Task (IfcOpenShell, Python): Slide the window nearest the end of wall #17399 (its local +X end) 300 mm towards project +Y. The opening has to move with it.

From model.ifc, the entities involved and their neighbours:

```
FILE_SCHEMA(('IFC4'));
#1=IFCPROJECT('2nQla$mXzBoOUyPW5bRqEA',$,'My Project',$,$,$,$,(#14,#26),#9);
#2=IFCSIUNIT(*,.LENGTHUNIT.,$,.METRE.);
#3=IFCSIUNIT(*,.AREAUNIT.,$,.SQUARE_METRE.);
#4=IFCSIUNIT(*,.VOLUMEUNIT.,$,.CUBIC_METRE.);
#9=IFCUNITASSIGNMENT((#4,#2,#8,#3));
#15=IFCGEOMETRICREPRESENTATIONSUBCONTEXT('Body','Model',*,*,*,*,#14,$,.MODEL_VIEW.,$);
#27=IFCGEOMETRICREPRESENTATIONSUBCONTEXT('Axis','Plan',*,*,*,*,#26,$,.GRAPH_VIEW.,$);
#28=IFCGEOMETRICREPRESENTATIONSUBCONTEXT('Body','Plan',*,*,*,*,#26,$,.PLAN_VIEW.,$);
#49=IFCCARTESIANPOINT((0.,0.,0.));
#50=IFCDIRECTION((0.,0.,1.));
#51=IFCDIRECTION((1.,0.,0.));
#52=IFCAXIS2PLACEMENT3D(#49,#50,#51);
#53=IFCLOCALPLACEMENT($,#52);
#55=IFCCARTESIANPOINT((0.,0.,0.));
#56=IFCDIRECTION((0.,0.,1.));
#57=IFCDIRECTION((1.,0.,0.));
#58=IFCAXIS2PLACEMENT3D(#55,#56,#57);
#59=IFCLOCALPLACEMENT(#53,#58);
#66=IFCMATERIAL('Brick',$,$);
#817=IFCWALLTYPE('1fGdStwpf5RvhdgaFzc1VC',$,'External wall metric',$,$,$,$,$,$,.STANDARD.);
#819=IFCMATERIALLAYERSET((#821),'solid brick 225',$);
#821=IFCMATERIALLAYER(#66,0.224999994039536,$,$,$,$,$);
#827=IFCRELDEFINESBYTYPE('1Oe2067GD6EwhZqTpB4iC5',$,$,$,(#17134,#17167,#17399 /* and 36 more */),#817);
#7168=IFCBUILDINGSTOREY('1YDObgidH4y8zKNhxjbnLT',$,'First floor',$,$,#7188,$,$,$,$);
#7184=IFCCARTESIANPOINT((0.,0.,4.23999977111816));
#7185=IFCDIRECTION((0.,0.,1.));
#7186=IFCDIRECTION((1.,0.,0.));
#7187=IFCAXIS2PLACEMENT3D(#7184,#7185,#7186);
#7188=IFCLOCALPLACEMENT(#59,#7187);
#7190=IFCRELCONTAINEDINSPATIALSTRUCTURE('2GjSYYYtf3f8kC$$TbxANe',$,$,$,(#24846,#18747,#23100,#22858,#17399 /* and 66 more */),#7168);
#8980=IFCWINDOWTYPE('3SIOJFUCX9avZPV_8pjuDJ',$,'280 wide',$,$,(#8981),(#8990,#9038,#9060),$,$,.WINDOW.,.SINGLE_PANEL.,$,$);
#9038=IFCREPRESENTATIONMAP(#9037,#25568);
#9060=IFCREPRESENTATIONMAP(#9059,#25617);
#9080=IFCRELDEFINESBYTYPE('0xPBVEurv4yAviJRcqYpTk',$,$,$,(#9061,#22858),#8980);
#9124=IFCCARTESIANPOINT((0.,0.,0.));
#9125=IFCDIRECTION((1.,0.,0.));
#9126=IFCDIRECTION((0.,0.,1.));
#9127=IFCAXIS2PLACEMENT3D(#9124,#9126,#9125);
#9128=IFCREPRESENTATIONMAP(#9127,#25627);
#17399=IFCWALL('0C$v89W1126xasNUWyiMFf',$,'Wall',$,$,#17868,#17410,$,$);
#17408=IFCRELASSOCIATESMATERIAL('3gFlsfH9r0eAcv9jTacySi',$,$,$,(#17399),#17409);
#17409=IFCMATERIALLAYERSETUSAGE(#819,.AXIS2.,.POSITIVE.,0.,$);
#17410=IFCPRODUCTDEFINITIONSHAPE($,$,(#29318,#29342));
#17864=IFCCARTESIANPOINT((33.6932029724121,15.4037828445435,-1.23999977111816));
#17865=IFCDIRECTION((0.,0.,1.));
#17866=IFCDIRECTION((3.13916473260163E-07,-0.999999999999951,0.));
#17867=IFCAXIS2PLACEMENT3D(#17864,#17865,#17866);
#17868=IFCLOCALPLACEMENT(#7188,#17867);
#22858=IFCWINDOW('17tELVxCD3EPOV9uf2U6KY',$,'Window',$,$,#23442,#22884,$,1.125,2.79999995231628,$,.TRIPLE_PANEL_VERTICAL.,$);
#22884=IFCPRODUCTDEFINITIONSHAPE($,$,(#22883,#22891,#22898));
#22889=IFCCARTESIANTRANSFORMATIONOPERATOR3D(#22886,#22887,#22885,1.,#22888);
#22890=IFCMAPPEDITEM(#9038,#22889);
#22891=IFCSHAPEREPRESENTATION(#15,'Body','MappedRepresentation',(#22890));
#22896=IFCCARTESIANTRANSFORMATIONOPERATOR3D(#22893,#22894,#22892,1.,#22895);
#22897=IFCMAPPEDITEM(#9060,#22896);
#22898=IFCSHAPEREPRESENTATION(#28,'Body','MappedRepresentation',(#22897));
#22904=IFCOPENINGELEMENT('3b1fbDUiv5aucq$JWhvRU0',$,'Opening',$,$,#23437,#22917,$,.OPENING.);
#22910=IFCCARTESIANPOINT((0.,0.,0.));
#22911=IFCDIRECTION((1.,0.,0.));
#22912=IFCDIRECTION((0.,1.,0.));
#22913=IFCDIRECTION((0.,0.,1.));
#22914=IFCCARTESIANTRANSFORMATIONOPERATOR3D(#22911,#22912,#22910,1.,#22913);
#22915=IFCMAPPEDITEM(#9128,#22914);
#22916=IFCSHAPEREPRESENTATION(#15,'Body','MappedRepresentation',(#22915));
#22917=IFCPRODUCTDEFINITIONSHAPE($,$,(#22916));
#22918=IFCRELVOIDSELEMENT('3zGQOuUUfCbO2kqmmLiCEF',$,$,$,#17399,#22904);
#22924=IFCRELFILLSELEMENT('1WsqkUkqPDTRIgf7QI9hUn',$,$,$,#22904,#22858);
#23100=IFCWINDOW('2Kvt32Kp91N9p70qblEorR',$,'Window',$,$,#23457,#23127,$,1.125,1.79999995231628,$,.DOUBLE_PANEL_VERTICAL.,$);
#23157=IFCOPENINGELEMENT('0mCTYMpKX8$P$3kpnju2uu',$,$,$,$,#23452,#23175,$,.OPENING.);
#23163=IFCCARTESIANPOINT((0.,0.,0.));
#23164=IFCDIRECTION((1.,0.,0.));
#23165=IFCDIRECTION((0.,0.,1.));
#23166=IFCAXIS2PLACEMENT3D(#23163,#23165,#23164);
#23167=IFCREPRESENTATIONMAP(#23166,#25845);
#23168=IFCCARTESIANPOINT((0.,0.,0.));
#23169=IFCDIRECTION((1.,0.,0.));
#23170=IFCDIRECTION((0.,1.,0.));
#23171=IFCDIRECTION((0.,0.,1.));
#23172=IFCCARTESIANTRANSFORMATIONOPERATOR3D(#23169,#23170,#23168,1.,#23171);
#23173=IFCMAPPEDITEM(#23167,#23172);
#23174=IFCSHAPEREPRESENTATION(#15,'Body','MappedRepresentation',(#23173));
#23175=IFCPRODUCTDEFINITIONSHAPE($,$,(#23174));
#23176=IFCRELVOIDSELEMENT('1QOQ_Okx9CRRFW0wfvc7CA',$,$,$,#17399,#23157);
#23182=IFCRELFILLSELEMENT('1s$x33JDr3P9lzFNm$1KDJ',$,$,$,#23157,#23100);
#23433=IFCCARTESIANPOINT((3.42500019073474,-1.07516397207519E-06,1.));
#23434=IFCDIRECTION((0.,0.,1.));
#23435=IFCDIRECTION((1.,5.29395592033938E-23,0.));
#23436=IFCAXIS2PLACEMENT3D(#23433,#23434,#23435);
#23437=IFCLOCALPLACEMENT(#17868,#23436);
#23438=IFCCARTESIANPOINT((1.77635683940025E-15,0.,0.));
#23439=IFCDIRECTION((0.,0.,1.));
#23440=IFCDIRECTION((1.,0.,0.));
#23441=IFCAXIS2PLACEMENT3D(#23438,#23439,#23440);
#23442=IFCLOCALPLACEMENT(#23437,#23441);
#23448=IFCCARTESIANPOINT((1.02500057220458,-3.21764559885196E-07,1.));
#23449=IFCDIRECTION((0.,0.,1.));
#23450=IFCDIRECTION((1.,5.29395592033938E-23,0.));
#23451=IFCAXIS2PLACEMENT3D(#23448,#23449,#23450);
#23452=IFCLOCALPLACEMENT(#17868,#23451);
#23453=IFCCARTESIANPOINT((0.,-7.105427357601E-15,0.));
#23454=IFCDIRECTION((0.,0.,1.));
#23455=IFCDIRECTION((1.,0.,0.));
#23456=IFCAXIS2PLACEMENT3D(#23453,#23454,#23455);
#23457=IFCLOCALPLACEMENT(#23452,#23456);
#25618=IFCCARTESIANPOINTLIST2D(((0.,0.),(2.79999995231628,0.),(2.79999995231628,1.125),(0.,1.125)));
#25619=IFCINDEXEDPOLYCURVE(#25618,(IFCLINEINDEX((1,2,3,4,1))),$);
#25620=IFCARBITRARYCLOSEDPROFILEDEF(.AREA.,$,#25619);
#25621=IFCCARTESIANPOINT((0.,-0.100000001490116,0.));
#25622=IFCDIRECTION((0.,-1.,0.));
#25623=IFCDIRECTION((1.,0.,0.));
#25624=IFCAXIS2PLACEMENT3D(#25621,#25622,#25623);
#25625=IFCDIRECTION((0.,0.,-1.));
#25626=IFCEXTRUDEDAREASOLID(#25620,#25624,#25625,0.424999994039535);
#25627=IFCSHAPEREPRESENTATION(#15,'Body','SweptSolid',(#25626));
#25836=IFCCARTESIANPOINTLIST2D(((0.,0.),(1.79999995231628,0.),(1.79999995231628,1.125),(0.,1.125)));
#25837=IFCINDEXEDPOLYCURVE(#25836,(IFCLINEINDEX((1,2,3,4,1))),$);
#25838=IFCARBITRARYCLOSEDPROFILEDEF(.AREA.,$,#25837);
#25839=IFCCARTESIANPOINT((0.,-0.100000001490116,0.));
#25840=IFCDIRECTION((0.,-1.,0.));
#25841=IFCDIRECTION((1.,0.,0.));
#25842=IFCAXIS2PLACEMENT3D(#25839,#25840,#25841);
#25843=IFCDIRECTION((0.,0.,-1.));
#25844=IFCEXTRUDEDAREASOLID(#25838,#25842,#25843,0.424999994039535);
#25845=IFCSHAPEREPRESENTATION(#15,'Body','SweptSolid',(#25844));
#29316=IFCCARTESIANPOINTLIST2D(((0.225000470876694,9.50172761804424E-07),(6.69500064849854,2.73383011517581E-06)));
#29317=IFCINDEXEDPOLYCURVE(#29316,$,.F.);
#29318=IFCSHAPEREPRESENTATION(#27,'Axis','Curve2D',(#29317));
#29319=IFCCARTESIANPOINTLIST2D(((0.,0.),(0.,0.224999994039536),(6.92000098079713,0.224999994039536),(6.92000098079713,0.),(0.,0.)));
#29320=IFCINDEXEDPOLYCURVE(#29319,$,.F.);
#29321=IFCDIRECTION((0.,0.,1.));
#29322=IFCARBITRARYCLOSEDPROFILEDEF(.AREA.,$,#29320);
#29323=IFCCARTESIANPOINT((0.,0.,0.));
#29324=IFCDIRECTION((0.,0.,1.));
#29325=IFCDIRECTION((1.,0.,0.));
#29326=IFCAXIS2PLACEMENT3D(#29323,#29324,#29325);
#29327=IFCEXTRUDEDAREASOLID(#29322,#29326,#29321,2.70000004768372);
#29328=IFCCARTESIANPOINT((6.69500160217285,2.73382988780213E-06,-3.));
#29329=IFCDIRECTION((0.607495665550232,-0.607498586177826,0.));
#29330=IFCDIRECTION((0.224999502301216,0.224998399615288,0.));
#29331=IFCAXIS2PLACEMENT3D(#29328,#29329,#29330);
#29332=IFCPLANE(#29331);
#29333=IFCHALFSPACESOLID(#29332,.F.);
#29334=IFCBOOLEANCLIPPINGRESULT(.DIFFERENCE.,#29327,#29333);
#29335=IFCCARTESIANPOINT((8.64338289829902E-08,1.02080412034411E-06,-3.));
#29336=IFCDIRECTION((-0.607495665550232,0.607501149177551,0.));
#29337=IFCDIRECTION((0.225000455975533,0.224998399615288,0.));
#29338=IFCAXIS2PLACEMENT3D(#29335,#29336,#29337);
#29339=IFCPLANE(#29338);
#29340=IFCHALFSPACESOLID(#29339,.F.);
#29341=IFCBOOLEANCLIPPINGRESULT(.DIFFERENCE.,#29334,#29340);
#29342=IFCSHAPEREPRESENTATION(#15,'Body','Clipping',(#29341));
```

```python
import ifcopenshell
import ifcopenshell.api.geometry
import ifcopenshell.util.placement

model = ifcopenshell.open("model.ifc")

window = model.by_guid("17tELVxCD3EPOV9uf2U6KY")
opening = window.FillsVoids[0].RelatingOpeningElement
wall = opening.VoidsElements[0].RelatingBuildingElement

wall_matrix = ifcopenshell.util.placement.get_local_placement(wall.ObjectPlacement)
shift = wall_matrix[:3, 0] * -0.3
before = ifcopenshell.util.placement.get_local_placement(window.ObjectPlacement)[:3, 3].copy()

# The window is placed relative to its opening, so it follows when the opening moves.
matrix = ifcopenshell.util.placement.get_local_placement(opening.ObjectPlacement)
matrix[:3, 3] += shift
ifcopenshell.api.geometry.edit_object_placement(
    model, product=opening, matrix=matrix, is_si=False, should_transform_children=True
)

after = ifcopenshell.util.placement.get_local_placement(window.ObjectPlacement)[:3, 3]
print("window moved by", (after - before).round(3) + 0.0)

model.write("model-out.ifc")
```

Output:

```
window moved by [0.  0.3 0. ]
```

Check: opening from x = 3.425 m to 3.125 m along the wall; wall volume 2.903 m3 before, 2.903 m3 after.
